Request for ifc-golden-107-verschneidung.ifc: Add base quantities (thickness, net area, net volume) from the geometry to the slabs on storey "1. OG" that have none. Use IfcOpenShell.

First a look at what the model holds.

```python
import ifcopenshell
import ifcopenshell.util.element
import ifcopenshell.util.unit

model = ifcopenshell.open("ifc-golden-107-verschneidung.ifc")
print(model.schema)
for unit_type in ("LENGTHUNIT", "AREAUNIT", "VOLUMEUNIT"):
    print(unit_type, ifcopenshell.util.unit.calculate_unit_scale(model, unit_type))
storey = next(s for s in model.by_type("IfcBuildingStorey") if s.Name == "1. OG")
slabs = [e for e in ifcopenshell.util.element.get_decomposition(storey) if e.is_a("IfcSlab")]
for e in sorted(slabs, key=lambda e: e.id()):
    print(e.id(), e.is_a(), e.Name, list(ifcopenshell.util.element.get_psets(e, qtos_only=True)), sep=" | ")
```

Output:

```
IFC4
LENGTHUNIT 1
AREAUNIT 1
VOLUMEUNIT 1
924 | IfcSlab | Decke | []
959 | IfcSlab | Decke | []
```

```python
import ifcopenshell
import ifcopenshell.api.pset
import ifcopenshell.geom
import ifcopenshell.util.element
import ifcopenshell.util.shape
import ifcopenshell.util.unit

model = ifcopenshell.open("ifc-golden-107-verschneidung.ifc")
unit_scale = ifcopenshell.util.unit.calculate_unit_scale(model)
area_scale = ifcopenshell.util.unit.calculate_unit_scale(model, "AREAUNIT")
volume_scale = ifcopenshell.util.unit.calculate_unit_scale(model, "VOLUMEUNIT")
settings = ifcopenshell.geom.settings()

storey = next(s for s in model.by_type("IfcBuildingStorey") if s.Name == "1. OG")
slabs = [e for e in ifcopenshell.util.element.get_decomposition(storey) if e.is_a("IfcSlab")]

for e in sorted(slabs, key=lambda e: e.id()):
    if ifcopenshell.util.element.get_psets(e, qtos_only=True, should_inherit=False):
        continue
    # Geometry comes back in metres, in the element's own axes.
    shape = ifcopenshell.geom.create_shape(settings, e)
    values = {
        "Width": ifcopenshell.util.shape.get_z(shape.geometry) / unit_scale,
        "NetArea": ifcopenshell.util.shape.get_footprint_area(shape.geometry) / area_scale,
        "NetVolume": ifcopenshell.util.shape.get_volume(shape.geometry) / volume_scale,
    }
    qto = ifcopenshell.api.pset.add_qto(model, product=e, name="Qto_SlabBaseQuantities")
    ifcopenshell.api.pset.edit_qto(model, qto=qto, properties=values)
    print(e.id(), {k: round(v, 3) for k, v in values.items()})

model.write("ifc-golden-107-verschneidung_rev.ifc")
```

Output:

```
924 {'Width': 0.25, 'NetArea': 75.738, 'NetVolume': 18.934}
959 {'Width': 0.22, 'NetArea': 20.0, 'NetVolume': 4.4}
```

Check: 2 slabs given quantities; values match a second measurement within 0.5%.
